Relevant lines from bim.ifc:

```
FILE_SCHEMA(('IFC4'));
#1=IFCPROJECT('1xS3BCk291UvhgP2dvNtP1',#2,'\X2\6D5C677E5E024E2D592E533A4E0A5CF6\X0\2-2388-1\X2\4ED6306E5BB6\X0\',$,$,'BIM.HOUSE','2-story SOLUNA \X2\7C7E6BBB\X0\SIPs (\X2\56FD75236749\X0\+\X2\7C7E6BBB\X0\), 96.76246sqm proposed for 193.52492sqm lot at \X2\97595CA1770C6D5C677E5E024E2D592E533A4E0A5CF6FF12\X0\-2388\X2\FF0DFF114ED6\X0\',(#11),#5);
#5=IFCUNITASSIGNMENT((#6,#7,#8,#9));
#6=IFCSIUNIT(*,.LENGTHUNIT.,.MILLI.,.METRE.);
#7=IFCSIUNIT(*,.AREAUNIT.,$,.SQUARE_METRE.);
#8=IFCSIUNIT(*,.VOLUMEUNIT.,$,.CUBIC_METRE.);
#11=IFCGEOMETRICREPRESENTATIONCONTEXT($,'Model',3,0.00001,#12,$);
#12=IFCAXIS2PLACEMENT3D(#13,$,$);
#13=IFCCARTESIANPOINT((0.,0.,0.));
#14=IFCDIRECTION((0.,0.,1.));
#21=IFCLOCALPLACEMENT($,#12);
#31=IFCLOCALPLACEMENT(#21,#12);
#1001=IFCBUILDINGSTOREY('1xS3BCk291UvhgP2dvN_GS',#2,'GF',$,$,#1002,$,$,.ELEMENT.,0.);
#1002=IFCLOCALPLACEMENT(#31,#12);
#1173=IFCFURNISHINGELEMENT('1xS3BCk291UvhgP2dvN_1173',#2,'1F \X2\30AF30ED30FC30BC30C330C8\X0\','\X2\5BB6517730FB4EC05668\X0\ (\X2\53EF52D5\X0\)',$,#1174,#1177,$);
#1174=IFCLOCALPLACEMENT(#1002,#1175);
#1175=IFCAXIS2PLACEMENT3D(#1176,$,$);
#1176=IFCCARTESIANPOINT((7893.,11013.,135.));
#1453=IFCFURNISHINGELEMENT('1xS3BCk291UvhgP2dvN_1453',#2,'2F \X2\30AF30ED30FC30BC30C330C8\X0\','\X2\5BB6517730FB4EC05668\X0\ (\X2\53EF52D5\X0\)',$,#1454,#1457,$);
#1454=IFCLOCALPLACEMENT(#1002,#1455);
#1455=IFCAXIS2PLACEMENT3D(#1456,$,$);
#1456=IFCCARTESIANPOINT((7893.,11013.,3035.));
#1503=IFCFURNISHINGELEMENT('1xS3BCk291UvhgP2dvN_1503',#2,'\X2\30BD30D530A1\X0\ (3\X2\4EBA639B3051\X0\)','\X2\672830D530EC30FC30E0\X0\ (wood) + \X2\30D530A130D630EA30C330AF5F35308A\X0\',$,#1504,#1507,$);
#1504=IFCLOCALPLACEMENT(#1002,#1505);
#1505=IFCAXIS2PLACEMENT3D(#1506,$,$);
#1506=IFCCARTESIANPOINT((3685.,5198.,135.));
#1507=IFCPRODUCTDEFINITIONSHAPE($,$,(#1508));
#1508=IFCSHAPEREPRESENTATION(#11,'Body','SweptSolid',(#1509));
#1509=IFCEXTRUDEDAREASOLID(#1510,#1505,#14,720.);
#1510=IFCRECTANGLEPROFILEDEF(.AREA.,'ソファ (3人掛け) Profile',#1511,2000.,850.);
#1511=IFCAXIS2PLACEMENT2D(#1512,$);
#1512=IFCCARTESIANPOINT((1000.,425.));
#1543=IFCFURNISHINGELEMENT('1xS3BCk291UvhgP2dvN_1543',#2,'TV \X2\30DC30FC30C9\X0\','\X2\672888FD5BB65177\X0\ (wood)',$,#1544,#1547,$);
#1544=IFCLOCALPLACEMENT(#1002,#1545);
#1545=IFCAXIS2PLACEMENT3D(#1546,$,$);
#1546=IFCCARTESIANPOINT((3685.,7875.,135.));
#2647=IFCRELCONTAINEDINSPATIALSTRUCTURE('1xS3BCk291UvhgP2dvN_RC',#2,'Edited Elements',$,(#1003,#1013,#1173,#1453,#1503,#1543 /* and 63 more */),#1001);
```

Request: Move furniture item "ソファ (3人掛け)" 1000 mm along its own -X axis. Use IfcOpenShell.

```python
import ifcopenshell
import ifcopenshell.api.geometry
import ifcopenshell.util.placement
import ifcopenshell.util.unit

model = ifcopenshell.open("bim.ifc")
unit_scale = ifcopenshell.util.unit.calculate_unit_scale(model)

item = model.by_guid("1xS3BCk291UvhgP2dvN_1503")
matrix = ifcopenshell.util.placement.get_local_placement(item.ObjectPlacement)
matrix[:3, 3] -= matrix[:3, 0] * 1 / unit_scale
ifcopenshell.api.geometry.edit_object_placement(model, product=item, matrix=matrix, is_si=False)

print(ifcopenshell.util.placement.get_local_placement(item.ObjectPlacement).round(3) + 0.0)

model.write("bim_updated.ifc")
```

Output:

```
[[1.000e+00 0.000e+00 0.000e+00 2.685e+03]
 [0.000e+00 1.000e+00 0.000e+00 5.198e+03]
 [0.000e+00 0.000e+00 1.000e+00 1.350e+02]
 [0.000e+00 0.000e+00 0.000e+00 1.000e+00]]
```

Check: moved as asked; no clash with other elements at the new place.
